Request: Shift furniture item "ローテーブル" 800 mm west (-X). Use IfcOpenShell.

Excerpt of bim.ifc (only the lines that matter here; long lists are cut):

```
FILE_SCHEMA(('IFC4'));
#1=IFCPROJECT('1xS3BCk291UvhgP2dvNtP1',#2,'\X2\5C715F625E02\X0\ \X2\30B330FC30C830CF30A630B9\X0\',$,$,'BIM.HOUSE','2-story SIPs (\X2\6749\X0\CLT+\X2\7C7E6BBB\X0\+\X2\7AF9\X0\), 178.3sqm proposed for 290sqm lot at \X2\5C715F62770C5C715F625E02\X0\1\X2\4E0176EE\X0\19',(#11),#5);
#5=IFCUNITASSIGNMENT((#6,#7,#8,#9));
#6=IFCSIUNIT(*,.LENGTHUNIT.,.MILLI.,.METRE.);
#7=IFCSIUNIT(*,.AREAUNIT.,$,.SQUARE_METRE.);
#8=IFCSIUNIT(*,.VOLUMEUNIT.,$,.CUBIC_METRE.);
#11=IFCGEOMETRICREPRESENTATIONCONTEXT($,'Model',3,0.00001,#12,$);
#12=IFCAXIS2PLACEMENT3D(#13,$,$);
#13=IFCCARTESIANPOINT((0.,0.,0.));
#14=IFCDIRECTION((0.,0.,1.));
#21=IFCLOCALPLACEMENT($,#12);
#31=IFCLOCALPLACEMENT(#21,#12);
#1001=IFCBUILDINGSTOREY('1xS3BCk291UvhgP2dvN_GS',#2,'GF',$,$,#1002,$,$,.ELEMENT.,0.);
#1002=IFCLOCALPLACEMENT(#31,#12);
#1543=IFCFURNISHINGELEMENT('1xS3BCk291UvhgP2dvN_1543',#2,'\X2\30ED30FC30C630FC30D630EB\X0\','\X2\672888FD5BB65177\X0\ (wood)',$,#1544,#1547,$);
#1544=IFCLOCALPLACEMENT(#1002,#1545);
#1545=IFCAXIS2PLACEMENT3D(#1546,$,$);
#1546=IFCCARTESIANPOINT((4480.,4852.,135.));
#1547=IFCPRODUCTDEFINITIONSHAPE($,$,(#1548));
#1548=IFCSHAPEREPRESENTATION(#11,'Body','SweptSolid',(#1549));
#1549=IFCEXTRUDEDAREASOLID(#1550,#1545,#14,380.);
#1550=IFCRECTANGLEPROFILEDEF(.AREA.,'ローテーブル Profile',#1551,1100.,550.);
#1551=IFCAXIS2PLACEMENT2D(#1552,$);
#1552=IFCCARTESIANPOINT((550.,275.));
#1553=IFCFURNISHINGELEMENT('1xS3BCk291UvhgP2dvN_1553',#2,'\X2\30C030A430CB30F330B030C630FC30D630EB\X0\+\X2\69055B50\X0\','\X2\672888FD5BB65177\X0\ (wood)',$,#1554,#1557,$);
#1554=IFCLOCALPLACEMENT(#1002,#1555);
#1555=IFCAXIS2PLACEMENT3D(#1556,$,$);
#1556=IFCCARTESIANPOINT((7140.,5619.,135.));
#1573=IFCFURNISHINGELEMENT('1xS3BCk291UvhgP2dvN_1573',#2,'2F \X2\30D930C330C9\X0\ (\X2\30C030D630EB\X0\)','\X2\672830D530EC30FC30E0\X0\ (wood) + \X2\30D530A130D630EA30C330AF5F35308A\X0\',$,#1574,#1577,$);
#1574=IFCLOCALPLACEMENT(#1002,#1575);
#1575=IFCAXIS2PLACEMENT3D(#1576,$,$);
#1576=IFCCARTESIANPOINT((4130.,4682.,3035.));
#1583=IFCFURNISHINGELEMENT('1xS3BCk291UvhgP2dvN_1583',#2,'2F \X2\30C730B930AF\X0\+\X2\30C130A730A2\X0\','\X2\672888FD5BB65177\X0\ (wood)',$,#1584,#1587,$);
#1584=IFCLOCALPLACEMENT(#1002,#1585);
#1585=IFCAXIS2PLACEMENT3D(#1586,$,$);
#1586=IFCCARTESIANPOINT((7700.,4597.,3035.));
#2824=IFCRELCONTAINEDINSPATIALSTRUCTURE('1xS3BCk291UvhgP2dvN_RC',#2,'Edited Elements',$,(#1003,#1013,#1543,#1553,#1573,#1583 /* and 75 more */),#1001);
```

```python
import ifcopenshell
import ifcopenshell.api.geometry
import ifcopenshell.util.placement
import ifcopenshell.util.unit

model = ifcopenshell.open("bim.ifc")
unit_scale = ifcopenshell.util.unit.calculate_unit_scale(model)

item = model.by_guid("1xS3BCk291UvhgP2dvN_1543")
matrix = ifcopenshell.util.placement.get_local_placement(item.ObjectPlacement)
matrix[0, 3] -= 0.8 / unit_scale
ifcopenshell.api.geometry.edit_object_placement(model, product=item, matrix=matrix, is_si=False)

print(ifcopenshell.util.placement.get_local_placement(item.ObjectPlacement).round(3) + 0.0)

model.write("bim_updated.ifc")
```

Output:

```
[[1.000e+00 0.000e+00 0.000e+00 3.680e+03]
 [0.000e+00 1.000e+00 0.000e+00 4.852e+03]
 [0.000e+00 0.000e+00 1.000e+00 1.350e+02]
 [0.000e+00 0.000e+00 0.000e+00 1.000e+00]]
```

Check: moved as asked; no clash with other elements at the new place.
